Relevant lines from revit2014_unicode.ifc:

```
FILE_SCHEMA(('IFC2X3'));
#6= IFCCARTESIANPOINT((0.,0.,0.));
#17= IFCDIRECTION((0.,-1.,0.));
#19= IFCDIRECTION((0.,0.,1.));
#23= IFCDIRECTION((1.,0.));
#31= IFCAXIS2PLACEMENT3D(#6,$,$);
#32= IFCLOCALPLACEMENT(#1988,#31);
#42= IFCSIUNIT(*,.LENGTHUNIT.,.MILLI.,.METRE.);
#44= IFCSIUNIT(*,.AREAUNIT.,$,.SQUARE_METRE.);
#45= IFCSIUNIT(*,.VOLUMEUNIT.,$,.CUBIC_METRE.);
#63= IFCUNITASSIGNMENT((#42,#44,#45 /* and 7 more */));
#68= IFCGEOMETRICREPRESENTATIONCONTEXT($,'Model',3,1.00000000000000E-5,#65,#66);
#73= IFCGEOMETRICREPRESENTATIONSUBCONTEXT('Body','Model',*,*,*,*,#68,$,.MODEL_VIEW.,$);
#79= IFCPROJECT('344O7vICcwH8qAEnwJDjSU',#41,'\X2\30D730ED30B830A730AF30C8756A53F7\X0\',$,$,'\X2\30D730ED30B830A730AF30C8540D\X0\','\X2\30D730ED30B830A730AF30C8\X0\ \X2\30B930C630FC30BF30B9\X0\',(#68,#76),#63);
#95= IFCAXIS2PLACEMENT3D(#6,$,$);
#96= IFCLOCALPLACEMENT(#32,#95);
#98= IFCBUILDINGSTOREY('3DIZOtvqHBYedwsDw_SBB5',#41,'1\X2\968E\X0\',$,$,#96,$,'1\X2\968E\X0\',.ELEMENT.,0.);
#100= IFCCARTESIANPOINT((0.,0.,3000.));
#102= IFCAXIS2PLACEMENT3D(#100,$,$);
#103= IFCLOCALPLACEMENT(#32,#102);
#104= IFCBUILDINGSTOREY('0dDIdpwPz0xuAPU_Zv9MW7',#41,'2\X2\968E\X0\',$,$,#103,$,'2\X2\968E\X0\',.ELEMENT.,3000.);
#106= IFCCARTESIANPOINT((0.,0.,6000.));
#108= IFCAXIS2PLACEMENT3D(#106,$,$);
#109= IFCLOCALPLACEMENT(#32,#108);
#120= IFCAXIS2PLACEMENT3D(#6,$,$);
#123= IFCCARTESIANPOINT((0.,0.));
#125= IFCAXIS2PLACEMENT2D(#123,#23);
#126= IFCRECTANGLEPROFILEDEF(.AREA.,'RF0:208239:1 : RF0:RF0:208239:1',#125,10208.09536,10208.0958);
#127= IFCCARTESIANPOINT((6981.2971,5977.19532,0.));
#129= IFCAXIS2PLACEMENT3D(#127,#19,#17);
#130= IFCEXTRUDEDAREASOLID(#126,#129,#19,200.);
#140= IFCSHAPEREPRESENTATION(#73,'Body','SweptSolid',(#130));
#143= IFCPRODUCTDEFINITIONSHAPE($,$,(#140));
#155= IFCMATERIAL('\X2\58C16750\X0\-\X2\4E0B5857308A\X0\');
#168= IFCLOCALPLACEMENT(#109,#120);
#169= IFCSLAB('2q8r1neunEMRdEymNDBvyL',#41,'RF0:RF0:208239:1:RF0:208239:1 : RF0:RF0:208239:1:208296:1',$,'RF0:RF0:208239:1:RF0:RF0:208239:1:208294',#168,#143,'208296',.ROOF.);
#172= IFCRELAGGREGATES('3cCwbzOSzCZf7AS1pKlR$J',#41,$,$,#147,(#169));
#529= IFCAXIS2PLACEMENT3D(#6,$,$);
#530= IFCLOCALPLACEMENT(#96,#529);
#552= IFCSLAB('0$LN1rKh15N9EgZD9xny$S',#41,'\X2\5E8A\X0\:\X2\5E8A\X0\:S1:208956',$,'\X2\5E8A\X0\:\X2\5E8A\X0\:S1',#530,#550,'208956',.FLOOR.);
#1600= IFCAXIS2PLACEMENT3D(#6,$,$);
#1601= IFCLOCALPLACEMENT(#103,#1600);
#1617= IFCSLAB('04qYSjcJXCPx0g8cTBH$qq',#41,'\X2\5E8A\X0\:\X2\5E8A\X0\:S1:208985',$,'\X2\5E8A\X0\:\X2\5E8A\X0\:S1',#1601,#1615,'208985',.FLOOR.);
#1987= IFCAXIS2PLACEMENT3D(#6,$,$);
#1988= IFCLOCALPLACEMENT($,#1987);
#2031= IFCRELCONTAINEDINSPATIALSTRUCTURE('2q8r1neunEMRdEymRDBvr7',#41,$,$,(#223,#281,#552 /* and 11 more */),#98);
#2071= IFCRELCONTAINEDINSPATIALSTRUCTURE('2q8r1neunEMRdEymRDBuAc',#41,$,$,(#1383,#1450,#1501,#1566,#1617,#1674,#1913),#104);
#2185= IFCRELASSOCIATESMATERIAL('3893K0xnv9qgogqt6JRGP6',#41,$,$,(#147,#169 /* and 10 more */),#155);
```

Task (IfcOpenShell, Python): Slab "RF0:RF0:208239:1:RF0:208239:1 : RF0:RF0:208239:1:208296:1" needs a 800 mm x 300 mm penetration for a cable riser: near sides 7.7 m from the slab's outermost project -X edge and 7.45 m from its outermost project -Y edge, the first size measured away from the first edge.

```python
import numpy as np
import ifcopenshell
import ifcopenshell.api.feature
import ifcopenshell.api.geometry
import ifcopenshell.api.root
import ifcopenshell.geom
import ifcopenshell.util.placement
import ifcopenshell.util.representation
import ifcopenshell.util.shape
import ifcopenshell.util.unit

model = ifcopenshell.open("revit2014_unicode.ifc")
unit_scale = ifcopenshell.util.unit.calculate_unit_scale(model)
settings = ifcopenshell.geom.settings()


def volume(element):
    """Net volume in cubic metres, openings subtracted."""
    shape = ifcopenshell.geom.create_shape(settings, element)
    return ifcopenshell.util.shape.get_volume(shape.geometry)


slab = model.by_guid("2q8r1neunEMRdEymNDBvyL")
before = volume(slab)

# Extent in the slab's own axes, in metres. The edges named are its -X and -Y sides.
slab_shape = ifcopenshell.geom.create_shape(settings, slab)
vertices = ifcopenshell.util.shape.get_vertices(slab_shape.geometry)
x_min, y_min, bottom = vertices.min(axis=0)
top = vertices[:, 2].max()

opening = ifcopenshell.api.root.create_entity(model, ifc_class="IfcOpeningElement", name="Cable riser opening")
context = ifcopenshell.util.representation.get_context(model, "Model", "Body", "MODEL_VIEW")
width, depth = 0.8, 0.3
outline = [(0.0, 0.0), (width, 0.0), (width, depth), (0.0, depth), (0.0, 0.0)]
# Overshoot both faces by 50 mm so the cut is clean.
shape = ifcopenshell.api.geometry.add_slab_representation(
    model, context=context, depth=top - bottom + 0.1, polyline=outline
)
ifcopenshell.api.geometry.assign_representation(model, product=opening, representation=shape)

matrix = ifcopenshell.util.placement.get_local_placement(slab.ObjectPlacement)
matrix[:, 3] = matrix @ np.append(np.array([x_min + 7.7, y_min + 7.45, bottom - 0.05]) / unit_scale, 1.0)
ifcopenshell.api.geometry.edit_object_placement(model, product=opening, matrix=matrix, is_si=False)
ifcopenshell.api.feature.add_feature(model, feature=opening, element=slab)

after = volume(slab)

print(f"slab volume {before:.3f} -> {after:.3f} m3")

model.write("revit2014_unicode_rev.ifc")
```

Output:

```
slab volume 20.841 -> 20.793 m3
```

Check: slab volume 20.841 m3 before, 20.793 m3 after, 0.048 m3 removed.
